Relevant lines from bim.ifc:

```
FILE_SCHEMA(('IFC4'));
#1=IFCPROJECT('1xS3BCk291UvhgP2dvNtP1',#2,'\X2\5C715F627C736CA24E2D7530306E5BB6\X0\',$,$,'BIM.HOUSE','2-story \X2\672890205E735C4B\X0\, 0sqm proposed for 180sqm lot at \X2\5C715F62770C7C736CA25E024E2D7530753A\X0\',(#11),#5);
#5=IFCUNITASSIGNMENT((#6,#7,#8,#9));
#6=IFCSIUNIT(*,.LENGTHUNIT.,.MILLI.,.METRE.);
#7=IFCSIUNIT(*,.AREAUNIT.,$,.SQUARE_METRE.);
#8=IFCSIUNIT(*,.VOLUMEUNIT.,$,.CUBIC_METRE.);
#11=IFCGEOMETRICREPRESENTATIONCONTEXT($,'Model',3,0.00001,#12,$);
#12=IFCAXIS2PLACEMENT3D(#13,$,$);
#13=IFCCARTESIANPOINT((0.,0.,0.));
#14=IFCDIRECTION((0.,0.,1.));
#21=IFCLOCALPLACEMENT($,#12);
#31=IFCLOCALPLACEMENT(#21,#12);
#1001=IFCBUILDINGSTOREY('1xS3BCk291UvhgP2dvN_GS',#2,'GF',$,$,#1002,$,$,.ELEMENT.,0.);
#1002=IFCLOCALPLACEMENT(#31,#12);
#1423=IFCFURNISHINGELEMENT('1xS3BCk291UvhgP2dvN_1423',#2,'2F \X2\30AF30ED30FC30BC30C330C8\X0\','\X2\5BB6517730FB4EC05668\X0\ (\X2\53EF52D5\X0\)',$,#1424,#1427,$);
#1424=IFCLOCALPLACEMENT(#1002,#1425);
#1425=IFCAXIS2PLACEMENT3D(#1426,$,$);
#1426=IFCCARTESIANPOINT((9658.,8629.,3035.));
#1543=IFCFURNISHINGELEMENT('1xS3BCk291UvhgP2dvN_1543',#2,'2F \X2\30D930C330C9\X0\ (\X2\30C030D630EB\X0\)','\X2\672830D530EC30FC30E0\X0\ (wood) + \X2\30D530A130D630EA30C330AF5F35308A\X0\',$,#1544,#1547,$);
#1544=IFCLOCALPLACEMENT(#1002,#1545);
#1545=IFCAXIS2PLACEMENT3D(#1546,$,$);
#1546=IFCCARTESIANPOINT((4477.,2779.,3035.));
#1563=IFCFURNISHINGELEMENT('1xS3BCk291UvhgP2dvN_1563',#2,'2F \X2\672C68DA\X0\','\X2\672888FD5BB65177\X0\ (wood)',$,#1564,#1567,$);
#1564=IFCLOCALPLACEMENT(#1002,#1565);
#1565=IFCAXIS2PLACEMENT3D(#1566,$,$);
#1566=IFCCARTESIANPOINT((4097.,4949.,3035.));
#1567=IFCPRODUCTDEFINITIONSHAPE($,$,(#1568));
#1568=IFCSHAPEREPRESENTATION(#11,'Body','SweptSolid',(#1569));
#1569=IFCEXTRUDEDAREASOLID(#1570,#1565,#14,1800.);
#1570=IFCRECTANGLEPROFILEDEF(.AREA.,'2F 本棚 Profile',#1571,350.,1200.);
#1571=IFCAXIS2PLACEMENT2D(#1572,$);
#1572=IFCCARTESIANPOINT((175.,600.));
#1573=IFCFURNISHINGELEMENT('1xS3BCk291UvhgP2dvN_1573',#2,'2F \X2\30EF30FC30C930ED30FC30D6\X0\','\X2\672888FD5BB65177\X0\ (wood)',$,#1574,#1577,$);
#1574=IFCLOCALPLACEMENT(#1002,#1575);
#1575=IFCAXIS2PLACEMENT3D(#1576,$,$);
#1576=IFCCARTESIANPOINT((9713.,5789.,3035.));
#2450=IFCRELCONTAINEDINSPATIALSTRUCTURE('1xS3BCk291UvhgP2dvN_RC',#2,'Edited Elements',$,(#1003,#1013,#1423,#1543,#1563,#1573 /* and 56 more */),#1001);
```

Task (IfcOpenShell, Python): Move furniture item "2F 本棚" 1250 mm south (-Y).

```python
import ifcopenshell
import ifcopenshell.api.geometry
import ifcopenshell.util.placement
import ifcopenshell.util.unit

model = ifcopenshell.open("bim.ifc")
unit_scale = ifcopenshell.util.unit.calculate_unit_scale(model)

item = model.by_guid("1xS3BCk291UvhgP2dvN_1563")
matrix = ifcopenshell.util.placement.get_local_placement(item.ObjectPlacement)
matrix[1, 3] -= 1.25 / unit_scale
ifcopenshell.api.geometry.edit_object_placement(model, product=item, matrix=matrix, is_si=False)

print(ifcopenshell.util.placement.get_local_placement(item.ObjectPlacement).round(3) + 0.0)

model.write("bim_edited.ifc")
```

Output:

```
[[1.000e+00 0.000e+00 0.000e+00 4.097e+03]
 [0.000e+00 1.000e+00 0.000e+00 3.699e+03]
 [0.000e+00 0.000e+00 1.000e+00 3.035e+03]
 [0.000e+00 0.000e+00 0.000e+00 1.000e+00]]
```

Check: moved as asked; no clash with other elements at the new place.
